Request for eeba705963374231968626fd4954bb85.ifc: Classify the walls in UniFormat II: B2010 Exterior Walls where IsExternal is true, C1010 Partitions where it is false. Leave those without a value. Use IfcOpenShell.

First a look at what the model holds.

```python
import ifcopenshell
import ifcopenshell.util.element

model = ifcopenshell.open("eeba705963374231968626fd4954bb85.ifc")
print(model.schema)
print("classifications:", [c.Name for c in model.by_type("IfcClassification")])
values = [ifcopenshell.util.element.get_pset(e, "Pset_WallCommon", "IsExternal") for e in model.by_type("IfcWall")]
for value in (True, False, None):
    print("IsExternal", value, values.count(value))
```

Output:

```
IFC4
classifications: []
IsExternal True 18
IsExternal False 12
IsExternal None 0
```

```python
import ifcopenshell
import ifcopenshell.api.classification
import ifcopenshell.util.element

model = ifcopenshell.open("eeba705963374231968626fd4954bb85.ifc")

system = ifcopenshell.api.classification.add_classification(model, classification="UniFormat II")

walls = model.by_type("IfcWall")
external = {e: ifcopenshell.util.element.get_pset(e, "Pset_WallCommon", "IsExternal") for e in walls}
for flag, code, name in ((True, "B2010", "Exterior Walls"), (False, "C1010", "Partitions")):
    products = [e for e in walls if external[e] is flag]
    ifcopenshell.api.classification.add_reference(
        model, products=products, classification=system, identification=code, name=name
    )
    print(code, len(products))

model.write("eeba705963374231968626fd4954bb85_edited.ifc")
```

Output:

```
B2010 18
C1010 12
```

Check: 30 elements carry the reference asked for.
